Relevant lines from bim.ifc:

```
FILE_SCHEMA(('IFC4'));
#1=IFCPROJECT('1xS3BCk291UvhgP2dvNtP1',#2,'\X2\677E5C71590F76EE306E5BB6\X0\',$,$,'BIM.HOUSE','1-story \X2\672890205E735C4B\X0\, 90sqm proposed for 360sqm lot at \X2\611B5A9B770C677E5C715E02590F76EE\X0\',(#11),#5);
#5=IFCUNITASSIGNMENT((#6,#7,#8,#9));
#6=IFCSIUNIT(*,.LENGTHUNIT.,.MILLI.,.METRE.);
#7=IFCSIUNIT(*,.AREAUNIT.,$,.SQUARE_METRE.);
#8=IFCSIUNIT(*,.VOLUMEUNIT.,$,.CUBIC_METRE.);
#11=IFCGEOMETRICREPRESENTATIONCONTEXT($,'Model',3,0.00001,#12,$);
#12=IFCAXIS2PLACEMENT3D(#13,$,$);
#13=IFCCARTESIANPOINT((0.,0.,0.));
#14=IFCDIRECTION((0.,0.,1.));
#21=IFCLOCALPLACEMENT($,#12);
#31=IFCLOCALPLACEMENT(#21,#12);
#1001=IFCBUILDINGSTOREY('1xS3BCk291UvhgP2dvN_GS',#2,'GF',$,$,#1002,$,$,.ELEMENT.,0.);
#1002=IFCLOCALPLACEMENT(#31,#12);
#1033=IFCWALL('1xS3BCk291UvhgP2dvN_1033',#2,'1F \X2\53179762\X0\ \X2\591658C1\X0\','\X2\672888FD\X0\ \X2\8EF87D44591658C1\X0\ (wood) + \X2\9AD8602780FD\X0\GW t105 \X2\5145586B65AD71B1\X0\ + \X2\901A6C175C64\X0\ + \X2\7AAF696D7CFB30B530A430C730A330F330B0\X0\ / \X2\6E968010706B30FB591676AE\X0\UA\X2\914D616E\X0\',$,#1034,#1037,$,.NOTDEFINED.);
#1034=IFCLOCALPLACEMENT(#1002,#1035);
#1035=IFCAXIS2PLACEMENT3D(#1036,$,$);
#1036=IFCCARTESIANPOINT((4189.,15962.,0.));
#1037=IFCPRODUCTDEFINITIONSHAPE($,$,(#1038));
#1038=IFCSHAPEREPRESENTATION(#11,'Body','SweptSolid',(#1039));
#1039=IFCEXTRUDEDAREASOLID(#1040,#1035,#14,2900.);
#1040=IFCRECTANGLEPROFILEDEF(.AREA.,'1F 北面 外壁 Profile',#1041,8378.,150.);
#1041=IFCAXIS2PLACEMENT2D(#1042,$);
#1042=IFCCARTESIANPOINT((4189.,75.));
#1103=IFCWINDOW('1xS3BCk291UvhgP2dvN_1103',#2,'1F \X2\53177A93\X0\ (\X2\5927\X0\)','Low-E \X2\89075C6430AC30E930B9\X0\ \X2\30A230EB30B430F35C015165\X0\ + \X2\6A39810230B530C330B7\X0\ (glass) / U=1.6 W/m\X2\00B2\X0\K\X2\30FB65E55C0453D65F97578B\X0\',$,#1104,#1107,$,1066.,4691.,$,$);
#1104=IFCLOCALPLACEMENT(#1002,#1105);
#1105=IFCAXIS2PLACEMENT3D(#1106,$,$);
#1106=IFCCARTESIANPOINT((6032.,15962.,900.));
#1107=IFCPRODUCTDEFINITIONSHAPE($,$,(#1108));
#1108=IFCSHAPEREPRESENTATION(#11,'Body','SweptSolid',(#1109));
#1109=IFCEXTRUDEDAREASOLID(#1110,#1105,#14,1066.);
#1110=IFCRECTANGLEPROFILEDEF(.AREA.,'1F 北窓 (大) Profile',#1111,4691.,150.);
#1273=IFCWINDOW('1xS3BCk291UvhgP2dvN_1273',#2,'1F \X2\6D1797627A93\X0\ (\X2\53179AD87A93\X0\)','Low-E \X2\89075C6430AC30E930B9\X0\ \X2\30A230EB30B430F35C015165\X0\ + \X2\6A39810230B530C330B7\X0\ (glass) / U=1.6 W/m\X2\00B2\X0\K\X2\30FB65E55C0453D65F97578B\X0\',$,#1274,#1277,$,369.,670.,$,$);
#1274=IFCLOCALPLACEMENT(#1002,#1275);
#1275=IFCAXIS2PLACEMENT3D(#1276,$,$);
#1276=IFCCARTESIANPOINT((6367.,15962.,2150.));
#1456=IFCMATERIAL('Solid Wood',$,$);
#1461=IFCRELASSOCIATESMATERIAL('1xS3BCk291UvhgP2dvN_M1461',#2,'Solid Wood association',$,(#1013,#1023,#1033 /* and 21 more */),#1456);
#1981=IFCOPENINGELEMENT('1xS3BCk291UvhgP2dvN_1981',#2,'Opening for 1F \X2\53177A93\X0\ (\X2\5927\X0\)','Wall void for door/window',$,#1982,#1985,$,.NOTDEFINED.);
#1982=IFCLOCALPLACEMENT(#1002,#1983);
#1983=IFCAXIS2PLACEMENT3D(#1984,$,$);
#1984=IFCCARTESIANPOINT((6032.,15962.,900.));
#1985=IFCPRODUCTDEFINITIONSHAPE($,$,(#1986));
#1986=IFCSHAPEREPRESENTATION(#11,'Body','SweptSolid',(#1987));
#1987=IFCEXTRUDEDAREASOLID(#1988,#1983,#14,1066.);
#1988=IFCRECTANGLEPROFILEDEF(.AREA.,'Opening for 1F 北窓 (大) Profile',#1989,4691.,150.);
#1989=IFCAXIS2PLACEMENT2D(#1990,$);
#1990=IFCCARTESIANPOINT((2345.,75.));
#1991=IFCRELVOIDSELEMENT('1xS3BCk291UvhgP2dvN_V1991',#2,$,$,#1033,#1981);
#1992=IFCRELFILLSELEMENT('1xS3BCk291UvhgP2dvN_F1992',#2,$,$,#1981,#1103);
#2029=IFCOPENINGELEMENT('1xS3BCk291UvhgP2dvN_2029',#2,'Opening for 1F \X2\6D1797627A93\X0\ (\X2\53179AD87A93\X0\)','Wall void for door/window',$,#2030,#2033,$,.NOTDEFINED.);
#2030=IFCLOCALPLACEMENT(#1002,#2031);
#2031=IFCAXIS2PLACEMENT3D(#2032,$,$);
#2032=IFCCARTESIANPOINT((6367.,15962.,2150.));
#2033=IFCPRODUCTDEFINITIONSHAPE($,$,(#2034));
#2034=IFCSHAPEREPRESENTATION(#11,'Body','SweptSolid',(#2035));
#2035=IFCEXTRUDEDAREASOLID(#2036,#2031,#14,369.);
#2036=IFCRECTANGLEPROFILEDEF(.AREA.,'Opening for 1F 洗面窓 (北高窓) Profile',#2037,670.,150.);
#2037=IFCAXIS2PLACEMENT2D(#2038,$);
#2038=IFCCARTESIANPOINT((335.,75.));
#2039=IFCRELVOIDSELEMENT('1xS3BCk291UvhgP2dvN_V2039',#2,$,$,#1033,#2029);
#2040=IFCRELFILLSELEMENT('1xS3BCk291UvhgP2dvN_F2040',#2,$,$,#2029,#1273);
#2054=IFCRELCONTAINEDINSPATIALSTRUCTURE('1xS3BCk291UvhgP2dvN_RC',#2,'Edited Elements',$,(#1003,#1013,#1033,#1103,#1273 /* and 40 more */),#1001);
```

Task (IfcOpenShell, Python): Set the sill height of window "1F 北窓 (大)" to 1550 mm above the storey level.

```python
import numpy as np
import ifcopenshell
import ifcopenshell.api.geometry
import ifcopenshell.geom
import ifcopenshell.util.element
import ifcopenshell.util.placement
import ifcopenshell.util.shape
import ifcopenshell.util.unit

model = ifcopenshell.open("bim.ifc")
unit_scale = ifcopenshell.util.unit.calculate_unit_scale(model)

window = model.by_id(1103)
opening = window.FillsVoids[0].RelatingOpeningElement
storey = ifcopenshell.util.element.get_container(window, ifc_class="IfcBuildingStorey")
level = ifcopenshell.util.placement.get_local_placement(storey.ObjectPlacement)[2, 3]

# The opening's origin need not be at the sill, so measure its lowest point.
shape = ifcopenshell.geom.create_shape(ifcopenshell.geom.settings(), opening)
bottom = ifcopenshell.util.shape.get_shape_bottom_elevation(shape, shape.geometry) / unit_scale
dz = level + 1.55 / unit_scale - bottom

shift = np.array([0.0, 0.0, dz])
# The window is not placed relative to its opening, so move both.
for product in (opening, window):
    matrix = ifcopenshell.util.placement.get_local_placement(product.ObjectPlacement)
    matrix[:3, 3] += shift
    ifcopenshell.api.geometry.edit_object_placement(model, product=product, matrix=matrix, is_si=False)

print(f"moved by {dz * unit_scale:+.3f} m")

model.write("bim-out.ifc")
```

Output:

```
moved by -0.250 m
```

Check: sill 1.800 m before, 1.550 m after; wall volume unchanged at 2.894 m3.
